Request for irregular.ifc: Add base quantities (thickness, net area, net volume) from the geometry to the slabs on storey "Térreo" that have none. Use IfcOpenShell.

First a look at what the model holds.

```python
import ifcopenshell
import ifcopenshell.util.element
import ifcopenshell.util.unit

model = ifcopenshell.open("irregular.ifc")
print(model.schema)
for unit_type in ("LENGTHUNIT", "AREAUNIT", "VOLUMEUNIT"):
    print(unit_type, ifcopenshell.util.unit.calculate_unit_scale(model, unit_type))
storey = next(s for s in model.by_type("IfcBuildingStorey") if s.Name == "Térreo")
slabs = [e for e in ifcopenshell.util.element.get_decomposition(storey) if e.is_a("IfcSlab")]
for e in sorted(slabs, key=lambda e: e.id()):
    print(e.id(), e.is_a(), e.Name, list(ifcopenshell.util.element.get_psets(e, qtos_only=True)), sep=" | ")
```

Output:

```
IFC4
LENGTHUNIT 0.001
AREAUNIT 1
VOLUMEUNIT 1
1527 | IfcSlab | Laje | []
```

```python
import ifcopenshell
import ifcopenshell.api.pset
import ifcopenshell.geom
import ifcopenshell.util.element
import ifcopenshell.util.shape
import ifcopenshell.util.unit

model = ifcopenshell.open("irregular.ifc")
unit_scale = ifcopenshell.util.unit.calculate_unit_scale(model)
area_scale = ifcopenshell.util.unit.calculate_unit_scale(model, "AREAUNIT")
volume_scale = ifcopenshell.util.unit.calculate_unit_scale(model, "VOLUMEUNIT")
settings = ifcopenshell.geom.settings()

storey = next(s for s in model.by_type("IfcBuildingStorey") if s.Name == "Térreo")
slabs = [e for e in ifcopenshell.util.element.get_decomposition(storey) if e.is_a("IfcSlab")]

for e in sorted(slabs, key=lambda e: e.id()):
    if ifcopenshell.util.element.get_psets(e, qtos_only=True, should_inherit=False):
        continue
    # Geometry comes back in metres, in the element's own axes.
    shape = ifcopenshell.geom.create_shape(settings, e)
    values = {
        "Width": ifcopenshell.util.shape.get_z(shape.geometry) / unit_scale,
        "NetArea": ifcopenshell.util.shape.get_footprint_area(shape.geometry) / area_scale,
        "NetVolume": ifcopenshell.util.shape.get_volume(shape.geometry) / volume_scale,
    }
    qto = ifcopenshell.api.pset.add_qto(model, product=e, name="Qto_SlabBaseQuantities")
    ifcopenshell.api.pset.edit_qto(model, qto=qto, properties=values)
    print(e.id(), {k: round(v, 3) for k, v in values.items()})

model.write("irregular_edited.ifc")
```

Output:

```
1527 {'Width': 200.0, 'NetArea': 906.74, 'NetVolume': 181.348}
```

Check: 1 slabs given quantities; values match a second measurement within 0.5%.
